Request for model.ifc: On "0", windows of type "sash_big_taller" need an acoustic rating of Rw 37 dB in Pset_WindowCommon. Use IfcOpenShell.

First a look at what the model holds.

```python
import ifcopenshell
import ifcopenshell.util.element

model = ifcopenshell.open("model.ifc")
print(model.schema)
storey = next(s for s in model.by_type("IfcBuildingStorey") if s.Name == "0")
windows = [e for e in ifcopenshell.util.element.get_decomposition(storey) if e.is_a("IfcWindow")]
seen = {}
for e in windows:
    element_type = ifcopenshell.util.element.get_type(e)
    key = (element_type.Name if element_type != e and element_type else None, ifcopenshell.util.element.get_pset(e, "Pset_WindowCommon", "AcousticRating"))
    seen[key] = seen.get(key, 0) + 1
for (name, value), count in sorted(seen.items(), key=str):
    print(count, "x", name, "|", value)
```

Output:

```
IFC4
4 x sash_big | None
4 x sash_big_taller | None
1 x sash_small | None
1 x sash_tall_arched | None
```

```python
import ifcopenshell
import ifcopenshell.api.pset
import ifcopenshell.util.element

model = ifcopenshell.open("model.ifc")

storey = next(s for s in model.by_type("IfcBuildingStorey") if s.Name == "0")
windows = [e for e in ifcopenshell.util.element.get_decomposition(storey) if e.is_a("IfcWindow")]

count = 0
for e in windows:
    element_type = ifcopenshell.util.element.get_type(e)
    if element_type in (None, e) or element_type.Name != "sash_big_taller":
        continue
    # add_pset returns the element's existing set when there is one.
    pset = ifcopenshell.api.pset.add_pset(model, product=e, name="Pset_WindowCommon")
    ifcopenshell.api.pset.edit_pset(model, pset=pset, properties={"AcousticRating": "Rw 37 dB"})
    count += 1

print(count, "windows updated")

model.write("model_updated.ifc")
```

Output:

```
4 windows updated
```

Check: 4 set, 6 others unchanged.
